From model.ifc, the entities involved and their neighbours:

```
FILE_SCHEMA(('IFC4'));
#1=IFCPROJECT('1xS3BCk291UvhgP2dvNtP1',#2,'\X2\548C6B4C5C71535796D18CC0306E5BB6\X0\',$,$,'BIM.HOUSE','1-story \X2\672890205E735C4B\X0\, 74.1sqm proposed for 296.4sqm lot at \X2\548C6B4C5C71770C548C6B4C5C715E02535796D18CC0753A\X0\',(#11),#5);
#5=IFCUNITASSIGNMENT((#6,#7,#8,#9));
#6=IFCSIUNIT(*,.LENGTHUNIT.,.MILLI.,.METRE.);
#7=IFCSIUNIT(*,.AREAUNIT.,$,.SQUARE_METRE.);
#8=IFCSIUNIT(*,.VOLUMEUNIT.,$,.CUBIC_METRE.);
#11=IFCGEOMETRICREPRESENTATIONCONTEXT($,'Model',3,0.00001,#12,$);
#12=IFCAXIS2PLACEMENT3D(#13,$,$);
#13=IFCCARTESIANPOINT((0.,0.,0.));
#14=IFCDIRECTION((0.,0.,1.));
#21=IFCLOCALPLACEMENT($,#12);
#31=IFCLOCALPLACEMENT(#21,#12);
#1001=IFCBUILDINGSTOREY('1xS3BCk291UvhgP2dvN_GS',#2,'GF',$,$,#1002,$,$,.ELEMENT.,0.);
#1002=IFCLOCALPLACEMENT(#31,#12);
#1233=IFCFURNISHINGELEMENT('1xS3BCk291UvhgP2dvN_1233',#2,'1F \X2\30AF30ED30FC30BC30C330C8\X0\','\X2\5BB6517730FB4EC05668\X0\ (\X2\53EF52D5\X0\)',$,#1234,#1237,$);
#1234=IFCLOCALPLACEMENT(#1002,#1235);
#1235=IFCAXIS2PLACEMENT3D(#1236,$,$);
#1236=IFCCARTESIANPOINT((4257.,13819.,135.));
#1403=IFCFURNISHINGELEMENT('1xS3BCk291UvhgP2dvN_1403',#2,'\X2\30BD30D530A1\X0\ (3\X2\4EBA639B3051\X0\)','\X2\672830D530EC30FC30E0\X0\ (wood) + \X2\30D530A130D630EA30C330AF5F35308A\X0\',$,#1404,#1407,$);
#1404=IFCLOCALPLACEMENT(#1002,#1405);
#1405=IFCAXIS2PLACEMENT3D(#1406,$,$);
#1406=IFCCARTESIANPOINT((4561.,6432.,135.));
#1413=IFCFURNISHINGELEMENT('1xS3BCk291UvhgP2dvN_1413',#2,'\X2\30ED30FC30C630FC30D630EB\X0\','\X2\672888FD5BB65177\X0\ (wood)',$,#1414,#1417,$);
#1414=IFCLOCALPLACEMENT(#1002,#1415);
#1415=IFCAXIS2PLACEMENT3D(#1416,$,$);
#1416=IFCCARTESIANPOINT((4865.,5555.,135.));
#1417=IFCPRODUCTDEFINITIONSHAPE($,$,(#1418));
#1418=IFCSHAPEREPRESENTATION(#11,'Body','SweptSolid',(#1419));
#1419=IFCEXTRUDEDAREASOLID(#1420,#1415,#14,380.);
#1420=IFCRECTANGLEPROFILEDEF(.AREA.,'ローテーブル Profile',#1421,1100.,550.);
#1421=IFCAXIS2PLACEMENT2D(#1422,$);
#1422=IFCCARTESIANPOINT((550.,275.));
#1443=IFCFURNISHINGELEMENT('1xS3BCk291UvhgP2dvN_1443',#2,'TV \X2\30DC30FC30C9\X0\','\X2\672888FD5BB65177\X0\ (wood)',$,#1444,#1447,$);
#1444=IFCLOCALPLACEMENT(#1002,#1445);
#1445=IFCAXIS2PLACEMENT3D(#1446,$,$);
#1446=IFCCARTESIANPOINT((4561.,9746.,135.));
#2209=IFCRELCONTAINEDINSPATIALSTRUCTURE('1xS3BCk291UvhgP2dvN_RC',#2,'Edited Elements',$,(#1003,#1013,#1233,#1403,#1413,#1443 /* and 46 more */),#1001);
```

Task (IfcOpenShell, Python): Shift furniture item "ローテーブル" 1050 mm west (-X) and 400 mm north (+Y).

```python
import ifcopenshell
import ifcopenshell.api.geometry
import ifcopenshell.util.placement

model = ifcopenshell.open("model.ifc")

item = model.by_id(1413)
matrix = ifcopenshell.util.placement.get_local_placement(item.ObjectPlacement)
matrix[0, 3] -= 1050.0
matrix[1, 3] += 400.0
ifcopenshell.api.geometry.edit_object_placement(model, product=item, matrix=matrix, is_si=False)

print(ifcopenshell.util.placement.get_local_placement(item.ObjectPlacement).round(3) + 0.0)

model.write("model_v2.ifc")
```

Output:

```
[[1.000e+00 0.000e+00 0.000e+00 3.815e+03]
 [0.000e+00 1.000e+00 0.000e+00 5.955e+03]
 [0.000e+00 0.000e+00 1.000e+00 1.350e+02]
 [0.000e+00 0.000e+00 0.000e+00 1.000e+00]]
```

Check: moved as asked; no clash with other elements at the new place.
